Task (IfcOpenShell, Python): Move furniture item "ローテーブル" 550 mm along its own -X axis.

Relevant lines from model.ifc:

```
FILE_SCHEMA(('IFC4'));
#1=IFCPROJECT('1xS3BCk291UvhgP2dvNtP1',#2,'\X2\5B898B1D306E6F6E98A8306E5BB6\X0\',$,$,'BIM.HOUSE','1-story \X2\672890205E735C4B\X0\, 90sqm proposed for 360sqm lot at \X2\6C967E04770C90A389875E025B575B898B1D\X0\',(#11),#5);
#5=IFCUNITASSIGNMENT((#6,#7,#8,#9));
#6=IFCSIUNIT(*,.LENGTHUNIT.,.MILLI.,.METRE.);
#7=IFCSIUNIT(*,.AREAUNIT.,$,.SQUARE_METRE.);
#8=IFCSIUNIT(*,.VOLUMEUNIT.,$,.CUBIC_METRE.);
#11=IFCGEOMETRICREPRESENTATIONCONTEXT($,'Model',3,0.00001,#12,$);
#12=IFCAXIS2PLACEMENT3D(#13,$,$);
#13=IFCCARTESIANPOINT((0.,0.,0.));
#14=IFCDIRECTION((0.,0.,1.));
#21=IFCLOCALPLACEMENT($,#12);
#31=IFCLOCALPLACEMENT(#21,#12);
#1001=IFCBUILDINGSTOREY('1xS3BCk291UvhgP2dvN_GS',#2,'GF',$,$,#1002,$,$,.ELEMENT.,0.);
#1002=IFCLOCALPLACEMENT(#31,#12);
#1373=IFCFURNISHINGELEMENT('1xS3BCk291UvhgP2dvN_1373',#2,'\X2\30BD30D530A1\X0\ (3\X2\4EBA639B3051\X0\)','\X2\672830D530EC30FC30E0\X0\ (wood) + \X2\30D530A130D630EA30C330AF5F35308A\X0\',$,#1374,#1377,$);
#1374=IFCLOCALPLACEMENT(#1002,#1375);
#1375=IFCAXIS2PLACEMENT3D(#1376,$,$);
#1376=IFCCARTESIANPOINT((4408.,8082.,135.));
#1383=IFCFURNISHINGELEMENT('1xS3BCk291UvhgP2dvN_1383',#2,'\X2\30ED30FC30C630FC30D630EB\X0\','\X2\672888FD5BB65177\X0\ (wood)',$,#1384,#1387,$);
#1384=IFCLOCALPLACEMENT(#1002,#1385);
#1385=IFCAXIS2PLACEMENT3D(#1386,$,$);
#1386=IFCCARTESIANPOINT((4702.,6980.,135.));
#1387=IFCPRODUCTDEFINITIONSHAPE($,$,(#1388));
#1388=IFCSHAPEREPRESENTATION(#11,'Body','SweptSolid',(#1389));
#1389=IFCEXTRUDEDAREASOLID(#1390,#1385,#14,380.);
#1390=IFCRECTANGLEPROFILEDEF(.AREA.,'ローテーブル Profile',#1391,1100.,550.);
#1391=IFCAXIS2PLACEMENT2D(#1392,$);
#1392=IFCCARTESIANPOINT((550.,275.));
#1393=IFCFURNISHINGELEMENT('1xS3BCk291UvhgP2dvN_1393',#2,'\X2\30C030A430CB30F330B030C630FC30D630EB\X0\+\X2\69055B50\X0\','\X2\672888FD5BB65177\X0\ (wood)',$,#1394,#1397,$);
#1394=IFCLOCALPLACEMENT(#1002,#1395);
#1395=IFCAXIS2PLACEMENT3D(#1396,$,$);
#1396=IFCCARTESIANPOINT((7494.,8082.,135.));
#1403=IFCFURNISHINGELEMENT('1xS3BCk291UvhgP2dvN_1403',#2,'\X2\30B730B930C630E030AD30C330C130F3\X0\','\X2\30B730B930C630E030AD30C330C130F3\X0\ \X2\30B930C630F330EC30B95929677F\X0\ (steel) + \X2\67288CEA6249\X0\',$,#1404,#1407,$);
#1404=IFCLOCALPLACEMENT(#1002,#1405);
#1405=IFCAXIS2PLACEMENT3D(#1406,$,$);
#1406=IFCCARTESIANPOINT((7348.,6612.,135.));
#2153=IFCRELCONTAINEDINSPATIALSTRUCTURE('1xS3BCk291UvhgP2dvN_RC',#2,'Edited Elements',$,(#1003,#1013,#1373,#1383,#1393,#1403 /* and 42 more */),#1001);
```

```python
import ifcopenshell
import ifcopenshell.api.geometry
import ifcopenshell.util.placement

model = ifcopenshell.open("model.ifc")

item = model.by_guid("1xS3BCk291UvhgP2dvN_1383")
matrix = ifcopenshell.util.placement.get_local_placement(item.ObjectPlacement)
matrix[:3, 3] -= matrix[:3, 0] * 550.0
ifcopenshell.api.geometry.edit_object_placement(model, product=item, matrix=matrix, is_si=False)

print(ifcopenshell.util.placement.get_local_placement(item.ObjectPlacement).round(3) + 0.0)

model.write("model_edited.ifc")
```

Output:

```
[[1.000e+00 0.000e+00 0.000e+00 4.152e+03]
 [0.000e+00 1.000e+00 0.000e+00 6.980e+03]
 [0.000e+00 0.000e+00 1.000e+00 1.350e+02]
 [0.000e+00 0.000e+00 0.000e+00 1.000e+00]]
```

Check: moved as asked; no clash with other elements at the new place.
